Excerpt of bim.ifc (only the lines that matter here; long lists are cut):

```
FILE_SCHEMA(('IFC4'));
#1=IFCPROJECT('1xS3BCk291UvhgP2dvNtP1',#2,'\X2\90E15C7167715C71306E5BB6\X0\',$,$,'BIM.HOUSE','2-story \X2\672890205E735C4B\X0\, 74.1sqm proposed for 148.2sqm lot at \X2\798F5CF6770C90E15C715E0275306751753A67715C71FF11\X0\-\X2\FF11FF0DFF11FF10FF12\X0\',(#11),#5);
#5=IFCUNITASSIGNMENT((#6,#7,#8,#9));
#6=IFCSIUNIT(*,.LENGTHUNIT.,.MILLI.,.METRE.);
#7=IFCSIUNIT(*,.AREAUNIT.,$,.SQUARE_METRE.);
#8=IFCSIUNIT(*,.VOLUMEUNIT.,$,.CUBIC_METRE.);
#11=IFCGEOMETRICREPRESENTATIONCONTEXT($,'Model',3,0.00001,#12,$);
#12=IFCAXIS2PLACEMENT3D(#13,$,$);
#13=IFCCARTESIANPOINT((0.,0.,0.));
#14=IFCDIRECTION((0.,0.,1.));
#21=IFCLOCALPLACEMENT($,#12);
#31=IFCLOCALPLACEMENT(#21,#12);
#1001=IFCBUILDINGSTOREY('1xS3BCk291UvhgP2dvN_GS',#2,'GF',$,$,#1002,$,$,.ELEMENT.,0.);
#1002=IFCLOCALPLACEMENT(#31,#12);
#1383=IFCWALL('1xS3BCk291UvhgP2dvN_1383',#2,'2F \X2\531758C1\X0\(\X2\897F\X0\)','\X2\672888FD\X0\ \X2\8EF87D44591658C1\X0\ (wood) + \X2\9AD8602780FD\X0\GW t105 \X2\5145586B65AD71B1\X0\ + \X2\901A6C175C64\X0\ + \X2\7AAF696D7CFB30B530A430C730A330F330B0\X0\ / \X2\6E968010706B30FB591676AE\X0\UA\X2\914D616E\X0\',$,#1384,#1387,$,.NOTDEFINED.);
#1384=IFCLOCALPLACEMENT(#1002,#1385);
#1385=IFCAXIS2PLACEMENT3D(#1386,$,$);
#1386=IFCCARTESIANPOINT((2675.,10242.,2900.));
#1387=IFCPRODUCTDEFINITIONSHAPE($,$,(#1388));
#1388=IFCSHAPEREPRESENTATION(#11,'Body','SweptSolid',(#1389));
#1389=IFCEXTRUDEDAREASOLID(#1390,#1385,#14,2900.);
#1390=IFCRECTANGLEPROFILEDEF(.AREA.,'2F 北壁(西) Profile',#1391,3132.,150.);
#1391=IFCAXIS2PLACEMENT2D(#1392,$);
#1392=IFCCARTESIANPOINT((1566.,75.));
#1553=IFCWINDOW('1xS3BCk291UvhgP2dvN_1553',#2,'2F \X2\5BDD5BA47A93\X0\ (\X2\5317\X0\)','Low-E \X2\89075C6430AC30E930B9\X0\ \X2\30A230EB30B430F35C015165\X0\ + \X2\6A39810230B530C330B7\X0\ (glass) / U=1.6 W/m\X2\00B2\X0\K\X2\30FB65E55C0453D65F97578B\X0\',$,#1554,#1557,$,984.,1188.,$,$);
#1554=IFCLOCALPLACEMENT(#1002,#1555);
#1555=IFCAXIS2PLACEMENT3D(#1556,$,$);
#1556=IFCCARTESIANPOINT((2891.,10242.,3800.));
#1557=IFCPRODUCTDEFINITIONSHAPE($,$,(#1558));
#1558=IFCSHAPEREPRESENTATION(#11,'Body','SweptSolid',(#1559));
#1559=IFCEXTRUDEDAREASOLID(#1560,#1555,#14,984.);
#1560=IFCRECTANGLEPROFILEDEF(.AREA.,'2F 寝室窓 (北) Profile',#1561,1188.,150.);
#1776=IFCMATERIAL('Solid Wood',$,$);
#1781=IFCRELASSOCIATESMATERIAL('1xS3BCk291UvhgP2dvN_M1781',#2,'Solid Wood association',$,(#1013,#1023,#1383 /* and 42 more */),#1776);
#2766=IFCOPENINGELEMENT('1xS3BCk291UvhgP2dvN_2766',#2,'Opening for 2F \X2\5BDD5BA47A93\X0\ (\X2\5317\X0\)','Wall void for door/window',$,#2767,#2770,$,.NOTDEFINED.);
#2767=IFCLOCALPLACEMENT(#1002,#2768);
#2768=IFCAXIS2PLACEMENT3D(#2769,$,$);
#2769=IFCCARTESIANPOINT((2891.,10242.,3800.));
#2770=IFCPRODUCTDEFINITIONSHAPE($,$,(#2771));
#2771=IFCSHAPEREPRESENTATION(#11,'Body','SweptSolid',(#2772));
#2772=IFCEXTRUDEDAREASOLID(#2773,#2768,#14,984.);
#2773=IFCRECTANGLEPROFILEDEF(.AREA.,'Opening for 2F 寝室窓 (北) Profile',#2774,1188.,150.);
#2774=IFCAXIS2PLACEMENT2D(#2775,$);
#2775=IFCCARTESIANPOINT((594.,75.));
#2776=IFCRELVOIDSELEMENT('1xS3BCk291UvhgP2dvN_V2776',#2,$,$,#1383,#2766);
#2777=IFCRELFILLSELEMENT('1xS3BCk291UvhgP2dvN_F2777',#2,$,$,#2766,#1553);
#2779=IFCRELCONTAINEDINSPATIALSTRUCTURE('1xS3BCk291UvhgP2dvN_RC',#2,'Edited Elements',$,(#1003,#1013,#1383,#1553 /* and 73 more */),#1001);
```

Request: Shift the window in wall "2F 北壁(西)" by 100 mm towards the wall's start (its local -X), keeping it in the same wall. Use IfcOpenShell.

```python
import ifcopenshell
import ifcopenshell.api.geometry
import ifcopenshell.util.placement
import ifcopenshell.util.unit

model = ifcopenshell.open("bim.ifc")
unit_scale = ifcopenshell.util.unit.calculate_unit_scale(model)

window = model.by_id(1553)
opening = window.FillsVoids[0].RelatingOpeningElement
wall = opening.VoidsElements[0].RelatingBuildingElement

wall_matrix = ifcopenshell.util.placement.get_local_placement(wall.ObjectPlacement)
shift = wall_matrix[:3, 0] * -0.1 / unit_scale
before = ifcopenshell.util.placement.get_local_placement(window.ObjectPlacement)[:3, 3].copy()

# The window is not placed relative to its opening, so move both.
for product in (opening, window):
    matrix = ifcopenshell.util.placement.get_local_placement(product.ObjectPlacement)
    matrix[:3, 3] += shift
    ifcopenshell.api.geometry.edit_object_placement(model, product=product, matrix=matrix, is_si=False)

after = ifcopenshell.util.placement.get_local_placement(window.ObjectPlacement)[:3, 3]
print("window moved by", (after - before).round(3) + 0.0)

model.write("bim_rev.ifc")
```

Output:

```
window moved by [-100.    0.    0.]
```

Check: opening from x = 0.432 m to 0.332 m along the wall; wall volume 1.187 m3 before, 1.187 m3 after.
